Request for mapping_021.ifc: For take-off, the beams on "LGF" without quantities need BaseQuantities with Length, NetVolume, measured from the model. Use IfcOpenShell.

First a look at what the model holds.

```python
import ifcopenshell
import ifcopenshell.util.element
import ifcopenshell.util.unit

model = ifcopenshell.open("mapping_021.ifc")
print(model.schema)
for unit_type in ("LENGTHUNIT", "AREAUNIT", "VOLUMEUNIT"):
    print(unit_type, ifcopenshell.util.unit.calculate_unit_scale(model, unit_type))
storey = next(s for s in model.by_type("IfcBuildingStorey") if s.Name == "LGF")
beams = [e for e in ifcopenshell.util.element.get_decomposition(storey) if e.is_a("IfcBeam")]
for e in sorted(beams, key=lambda e: e.id()):
    print(e.id(), e.is_a(), e.Name, list(ifcopenshell.util.element.get_psets(e, qtos_only=True)), sep=" | ")
```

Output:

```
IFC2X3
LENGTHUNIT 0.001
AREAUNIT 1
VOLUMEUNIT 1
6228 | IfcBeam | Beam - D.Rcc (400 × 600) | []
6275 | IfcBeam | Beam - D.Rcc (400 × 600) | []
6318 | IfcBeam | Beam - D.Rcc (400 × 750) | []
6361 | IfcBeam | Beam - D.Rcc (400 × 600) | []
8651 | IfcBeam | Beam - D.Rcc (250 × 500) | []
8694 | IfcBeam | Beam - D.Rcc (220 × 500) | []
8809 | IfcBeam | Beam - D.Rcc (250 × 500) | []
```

```python
import ifcopenshell
import ifcopenshell.api.pset
import ifcopenshell.geom
import ifcopenshell.util.element
import ifcopenshell.util.shape
import ifcopenshell.util.unit

model = ifcopenshell.open("mapping_021.ifc")
unit_scale = ifcopenshell.util.unit.calculate_unit_scale(model)
volume_scale = ifcopenshell.util.unit.calculate_unit_scale(model, "VOLUMEUNIT")
settings = ifcopenshell.geom.settings()

storey = next(s for s in model.by_type("IfcBuildingStorey") if s.Name == "LGF")
beams = [e for e in ifcopenshell.util.element.get_decomposition(storey) if e.is_a("IfcBeam")]

for e in sorted(beams, key=lambda e: e.id()):
    if ifcopenshell.util.element.get_psets(e, qtos_only=True, should_inherit=False):
        continue
    # Geometry comes back in metres, in the element's own axes.
    shape = ifcopenshell.geom.create_shape(settings, e)
    values = {
        "Length": ifcopenshell.util.shape.get_max_xyz(shape.geometry) / unit_scale,
        "NetVolume": ifcopenshell.util.shape.get_volume(shape.geometry) / volume_scale,
    }
    qto = ifcopenshell.api.pset.add_qto(model, product=e, name="BaseQuantities")
    ifcopenshell.api.pset.edit_qto(model, qto=qto, properties=values)
    print(e.id(), {k: round(v, 3) for k, v in values.items()})

model.write("mapping_021_edited.ifc")
```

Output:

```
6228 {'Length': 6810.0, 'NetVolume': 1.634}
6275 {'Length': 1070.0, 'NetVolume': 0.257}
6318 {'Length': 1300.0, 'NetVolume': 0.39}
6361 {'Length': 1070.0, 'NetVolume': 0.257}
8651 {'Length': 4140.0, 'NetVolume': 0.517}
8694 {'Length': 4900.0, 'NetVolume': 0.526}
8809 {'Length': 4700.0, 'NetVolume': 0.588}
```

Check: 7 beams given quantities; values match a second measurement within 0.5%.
